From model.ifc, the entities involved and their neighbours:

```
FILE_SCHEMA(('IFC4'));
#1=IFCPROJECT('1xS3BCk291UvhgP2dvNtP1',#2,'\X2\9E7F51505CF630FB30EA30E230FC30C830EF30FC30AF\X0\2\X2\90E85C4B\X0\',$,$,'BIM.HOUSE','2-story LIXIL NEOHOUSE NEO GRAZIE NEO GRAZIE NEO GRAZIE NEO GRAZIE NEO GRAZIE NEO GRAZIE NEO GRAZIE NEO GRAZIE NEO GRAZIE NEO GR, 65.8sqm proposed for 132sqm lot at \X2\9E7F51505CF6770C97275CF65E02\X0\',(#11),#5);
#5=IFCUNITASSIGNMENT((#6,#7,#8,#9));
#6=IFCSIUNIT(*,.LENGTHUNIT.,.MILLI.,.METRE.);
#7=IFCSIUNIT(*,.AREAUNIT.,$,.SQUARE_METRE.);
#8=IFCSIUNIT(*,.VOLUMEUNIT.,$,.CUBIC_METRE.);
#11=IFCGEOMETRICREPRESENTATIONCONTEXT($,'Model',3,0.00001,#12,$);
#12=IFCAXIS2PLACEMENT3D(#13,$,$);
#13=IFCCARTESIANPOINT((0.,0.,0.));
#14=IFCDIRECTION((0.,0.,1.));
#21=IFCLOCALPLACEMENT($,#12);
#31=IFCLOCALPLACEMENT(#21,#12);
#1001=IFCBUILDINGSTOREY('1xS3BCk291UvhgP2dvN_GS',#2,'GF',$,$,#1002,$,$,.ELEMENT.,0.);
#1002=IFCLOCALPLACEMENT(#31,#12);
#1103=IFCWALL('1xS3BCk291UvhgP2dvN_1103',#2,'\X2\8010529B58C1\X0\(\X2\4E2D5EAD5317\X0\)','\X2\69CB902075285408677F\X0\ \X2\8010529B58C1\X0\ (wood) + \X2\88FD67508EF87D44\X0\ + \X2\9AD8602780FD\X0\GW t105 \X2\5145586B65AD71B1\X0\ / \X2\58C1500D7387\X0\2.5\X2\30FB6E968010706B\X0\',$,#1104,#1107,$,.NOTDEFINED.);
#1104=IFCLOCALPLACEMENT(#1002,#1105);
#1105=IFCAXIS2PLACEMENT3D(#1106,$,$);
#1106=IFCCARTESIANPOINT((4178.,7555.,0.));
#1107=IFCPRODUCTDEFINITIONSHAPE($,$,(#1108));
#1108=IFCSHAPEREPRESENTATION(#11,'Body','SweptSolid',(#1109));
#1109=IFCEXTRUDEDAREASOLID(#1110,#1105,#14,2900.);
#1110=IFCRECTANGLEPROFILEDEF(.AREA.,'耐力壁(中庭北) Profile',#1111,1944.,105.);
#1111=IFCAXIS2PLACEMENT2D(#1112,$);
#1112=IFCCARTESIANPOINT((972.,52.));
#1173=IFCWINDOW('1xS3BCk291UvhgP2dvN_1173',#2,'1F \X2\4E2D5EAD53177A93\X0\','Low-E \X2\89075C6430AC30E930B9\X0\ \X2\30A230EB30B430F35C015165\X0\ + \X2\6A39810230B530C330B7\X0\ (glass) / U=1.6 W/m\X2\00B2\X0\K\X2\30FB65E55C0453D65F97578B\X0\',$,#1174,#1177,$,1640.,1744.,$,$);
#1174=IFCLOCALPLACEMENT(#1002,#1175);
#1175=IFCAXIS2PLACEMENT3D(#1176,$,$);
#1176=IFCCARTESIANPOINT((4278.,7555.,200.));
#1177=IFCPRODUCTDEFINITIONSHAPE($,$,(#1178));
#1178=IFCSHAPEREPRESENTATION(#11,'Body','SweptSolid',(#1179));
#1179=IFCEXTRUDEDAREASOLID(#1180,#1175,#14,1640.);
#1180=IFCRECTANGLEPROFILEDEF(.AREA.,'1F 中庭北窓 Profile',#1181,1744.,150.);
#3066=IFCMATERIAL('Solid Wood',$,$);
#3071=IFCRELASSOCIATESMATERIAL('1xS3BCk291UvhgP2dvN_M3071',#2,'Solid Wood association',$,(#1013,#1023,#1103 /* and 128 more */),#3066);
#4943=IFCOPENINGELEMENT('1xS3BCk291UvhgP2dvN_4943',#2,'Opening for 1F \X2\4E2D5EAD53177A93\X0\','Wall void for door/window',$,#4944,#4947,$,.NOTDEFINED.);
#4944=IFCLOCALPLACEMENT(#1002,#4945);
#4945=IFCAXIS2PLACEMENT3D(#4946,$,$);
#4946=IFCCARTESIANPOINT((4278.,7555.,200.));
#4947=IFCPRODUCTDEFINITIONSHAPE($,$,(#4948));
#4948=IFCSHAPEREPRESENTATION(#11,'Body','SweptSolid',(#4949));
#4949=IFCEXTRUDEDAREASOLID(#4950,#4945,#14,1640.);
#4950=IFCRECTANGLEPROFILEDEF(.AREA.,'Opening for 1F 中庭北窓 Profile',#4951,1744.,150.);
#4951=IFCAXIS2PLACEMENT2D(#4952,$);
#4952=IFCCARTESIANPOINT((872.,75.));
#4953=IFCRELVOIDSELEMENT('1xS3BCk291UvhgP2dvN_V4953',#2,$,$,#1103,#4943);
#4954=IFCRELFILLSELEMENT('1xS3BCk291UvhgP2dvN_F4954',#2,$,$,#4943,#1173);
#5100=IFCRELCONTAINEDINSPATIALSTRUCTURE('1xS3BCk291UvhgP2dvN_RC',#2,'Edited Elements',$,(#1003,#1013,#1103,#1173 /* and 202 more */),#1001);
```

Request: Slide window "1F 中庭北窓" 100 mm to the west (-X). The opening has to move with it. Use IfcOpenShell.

```python
import ifcopenshell
import ifcopenshell.api.geometry
import ifcopenshell.util.placement

model = ifcopenshell.open("model.ifc")

window = model.by_guid("1xS3BCk291UvhgP2dvN_1173")
opening = window.FillsVoids[0].RelatingOpeningElement
wall = opening.VoidsElements[0].RelatingBuildingElement

wall_matrix = ifcopenshell.util.placement.get_local_placement(wall.ObjectPlacement)
shift = wall_matrix[:3, 0] * -100.0
before = ifcopenshell.util.placement.get_local_placement(window.ObjectPlacement)[:3, 3].copy()

# The window is not placed relative to its opening, so move both.
for product in (opening, window):
    matrix = ifcopenshell.util.placement.get_local_placement(product.ObjectPlacement)
    matrix[:3, 3] += shift
    ifcopenshell.api.geometry.edit_object_placement(model, product=product, matrix=matrix, is_si=False)

after = ifcopenshell.util.placement.get_local_placement(window.ObjectPlacement)[:3, 3]
print("window moved by", (after - before).round(3) + 0.0)

model.write("model_edited.ifc")
```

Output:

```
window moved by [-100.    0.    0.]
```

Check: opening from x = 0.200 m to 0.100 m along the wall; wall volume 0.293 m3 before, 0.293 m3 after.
